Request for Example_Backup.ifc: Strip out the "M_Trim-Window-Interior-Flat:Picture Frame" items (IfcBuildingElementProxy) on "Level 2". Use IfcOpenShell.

First a look at what the model holds.

```python
import ifcopenshell
import ifcopenshell.util.element

model = ifcopenshell.open("Example_Backup.ifc")
print(model.schema)
storey = next(s for s in model.by_type("IfcBuildingStorey") if s.Name == "Level 2")
proxies = [e for e in ifcopenshell.util.element.get_decomposition(storey) if e.is_a("IfcBuildingElementProxy")]
seen = {}
for e in proxies:
    element_type = ifcopenshell.util.element.get_type(e)
    name = element_type.Name if element_type not in (None, e) else None
    seen[name] = seen.get(name, 0) + 1
for name, count in sorted(seen.items(), key=str):
    print(count, "x", name)
```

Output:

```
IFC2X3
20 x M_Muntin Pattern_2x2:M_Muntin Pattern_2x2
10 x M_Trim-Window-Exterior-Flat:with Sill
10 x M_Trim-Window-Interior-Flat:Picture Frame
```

```python
import ifcopenshell
import ifcopenshell.api.root
import ifcopenshell.util.element

model = ifcopenshell.open("Example_Backup.ifc")

storey = next(s for s in model.by_type("IfcBuildingStorey") if s.Name == "Level 2")
proxies = [e for e in ifcopenshell.util.element.get_decomposition(storey) if e.is_a("IfcBuildingElementProxy")]
targets = [e for e in proxies if (t := ifcopenshell.util.element.get_type(e)) not in (None, e) and t.Name == "M_Trim-Window-Interior-Flat:Picture Frame"]

for e in targets:
    ifcopenshell.api.root.remove_product(model, product=e)
print(len(targets), "removed")

model.write("Example_Backup_v2.ifc")
```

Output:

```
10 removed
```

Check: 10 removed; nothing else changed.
